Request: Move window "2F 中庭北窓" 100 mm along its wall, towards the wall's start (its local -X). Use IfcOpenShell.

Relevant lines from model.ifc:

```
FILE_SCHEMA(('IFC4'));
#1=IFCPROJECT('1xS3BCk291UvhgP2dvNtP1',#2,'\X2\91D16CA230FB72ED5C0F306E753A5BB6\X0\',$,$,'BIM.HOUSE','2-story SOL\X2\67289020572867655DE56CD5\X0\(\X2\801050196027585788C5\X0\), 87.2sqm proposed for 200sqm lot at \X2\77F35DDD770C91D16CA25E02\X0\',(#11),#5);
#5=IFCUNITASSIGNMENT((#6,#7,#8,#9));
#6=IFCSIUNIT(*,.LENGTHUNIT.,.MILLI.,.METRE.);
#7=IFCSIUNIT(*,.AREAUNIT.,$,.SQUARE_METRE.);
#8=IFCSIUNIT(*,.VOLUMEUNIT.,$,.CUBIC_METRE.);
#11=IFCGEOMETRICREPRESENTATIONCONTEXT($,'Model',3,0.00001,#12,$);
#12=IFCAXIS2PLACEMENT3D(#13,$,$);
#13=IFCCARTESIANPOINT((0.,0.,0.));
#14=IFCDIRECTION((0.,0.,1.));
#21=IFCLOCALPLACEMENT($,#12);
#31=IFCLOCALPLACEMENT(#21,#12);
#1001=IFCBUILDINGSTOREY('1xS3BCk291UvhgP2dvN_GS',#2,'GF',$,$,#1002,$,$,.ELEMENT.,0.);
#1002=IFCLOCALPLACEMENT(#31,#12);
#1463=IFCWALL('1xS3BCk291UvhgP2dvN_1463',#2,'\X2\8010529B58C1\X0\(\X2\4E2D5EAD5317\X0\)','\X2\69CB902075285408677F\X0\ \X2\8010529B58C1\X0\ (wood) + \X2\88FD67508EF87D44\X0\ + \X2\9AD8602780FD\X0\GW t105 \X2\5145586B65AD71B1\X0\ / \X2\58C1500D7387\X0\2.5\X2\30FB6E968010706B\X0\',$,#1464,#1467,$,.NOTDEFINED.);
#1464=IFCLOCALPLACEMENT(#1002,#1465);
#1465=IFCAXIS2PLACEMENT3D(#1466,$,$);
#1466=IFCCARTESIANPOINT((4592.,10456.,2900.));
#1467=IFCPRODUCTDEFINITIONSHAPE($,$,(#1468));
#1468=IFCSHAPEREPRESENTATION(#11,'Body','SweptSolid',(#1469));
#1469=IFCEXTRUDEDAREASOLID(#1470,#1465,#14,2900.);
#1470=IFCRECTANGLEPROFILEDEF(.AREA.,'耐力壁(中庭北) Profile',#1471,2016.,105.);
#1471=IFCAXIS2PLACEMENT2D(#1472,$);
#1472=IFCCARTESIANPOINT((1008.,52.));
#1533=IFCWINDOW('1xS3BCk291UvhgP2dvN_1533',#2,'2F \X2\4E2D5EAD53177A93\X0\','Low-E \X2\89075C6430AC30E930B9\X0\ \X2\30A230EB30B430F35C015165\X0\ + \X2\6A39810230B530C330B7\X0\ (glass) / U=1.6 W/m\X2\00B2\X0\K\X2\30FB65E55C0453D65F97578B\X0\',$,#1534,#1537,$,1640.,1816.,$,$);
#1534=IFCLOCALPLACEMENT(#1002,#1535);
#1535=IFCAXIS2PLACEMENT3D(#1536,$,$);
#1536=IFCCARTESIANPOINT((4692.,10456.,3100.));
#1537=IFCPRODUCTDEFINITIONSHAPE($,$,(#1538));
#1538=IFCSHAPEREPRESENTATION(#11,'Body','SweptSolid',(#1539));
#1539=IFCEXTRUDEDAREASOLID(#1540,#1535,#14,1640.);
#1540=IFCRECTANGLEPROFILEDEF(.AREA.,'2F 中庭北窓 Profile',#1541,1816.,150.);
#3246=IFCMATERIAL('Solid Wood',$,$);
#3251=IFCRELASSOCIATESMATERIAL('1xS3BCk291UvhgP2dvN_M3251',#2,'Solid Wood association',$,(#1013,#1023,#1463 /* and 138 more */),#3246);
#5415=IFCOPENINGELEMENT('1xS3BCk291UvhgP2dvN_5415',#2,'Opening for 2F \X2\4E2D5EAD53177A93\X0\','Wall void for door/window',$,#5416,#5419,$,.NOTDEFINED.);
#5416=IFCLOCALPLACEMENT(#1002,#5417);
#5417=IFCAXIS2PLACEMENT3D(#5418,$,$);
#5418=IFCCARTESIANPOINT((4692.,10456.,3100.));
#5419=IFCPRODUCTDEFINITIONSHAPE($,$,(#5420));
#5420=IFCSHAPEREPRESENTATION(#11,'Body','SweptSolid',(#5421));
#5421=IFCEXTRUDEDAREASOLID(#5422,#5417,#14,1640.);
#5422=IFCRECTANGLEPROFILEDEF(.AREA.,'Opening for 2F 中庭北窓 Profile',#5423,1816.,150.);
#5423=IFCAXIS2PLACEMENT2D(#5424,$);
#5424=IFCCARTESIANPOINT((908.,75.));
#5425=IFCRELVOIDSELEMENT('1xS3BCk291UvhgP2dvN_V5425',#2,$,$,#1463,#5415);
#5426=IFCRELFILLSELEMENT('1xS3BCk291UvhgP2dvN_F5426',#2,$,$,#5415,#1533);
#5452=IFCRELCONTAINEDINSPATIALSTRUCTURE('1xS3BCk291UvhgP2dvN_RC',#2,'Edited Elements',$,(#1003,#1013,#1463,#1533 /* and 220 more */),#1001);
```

```python
import ifcopenshell
import ifcopenshell.api.geometry
import ifcopenshell.util.placement

model = ifcopenshell.open("model.ifc")

window = model.by_id(1533)
opening = window.FillsVoids[0].RelatingOpeningElement
wall = opening.VoidsElements[0].RelatingBuildingElement

wall_matrix = ifcopenshell.util.placement.get_local_placement(wall.ObjectPlacement)
shift = wall_matrix[:3, 0] * -100.0
before = ifcopenshell.util.placement.get_local_placement(window.ObjectPlacement)[:3, 3].copy()

# The window is not placed relative to its opening, so move both.
for product in (opening, window):
    matrix = ifcopenshell.util.placement.get_local_placement(product.ObjectPlacement)
    matrix[:3, 3] += shift
    ifcopenshell.api.geometry.edit_object_placement(model, product=product, matrix=matrix, is_si=False)

after = ifcopenshell.util.placement.get_local_placement(window.ObjectPlacement)[:3, 3]
print("window moved by", (after - before).round(3) + 0.0)

model.write("model_rev.ifc")
```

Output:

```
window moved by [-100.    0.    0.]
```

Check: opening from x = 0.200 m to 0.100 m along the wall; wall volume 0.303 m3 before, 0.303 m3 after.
